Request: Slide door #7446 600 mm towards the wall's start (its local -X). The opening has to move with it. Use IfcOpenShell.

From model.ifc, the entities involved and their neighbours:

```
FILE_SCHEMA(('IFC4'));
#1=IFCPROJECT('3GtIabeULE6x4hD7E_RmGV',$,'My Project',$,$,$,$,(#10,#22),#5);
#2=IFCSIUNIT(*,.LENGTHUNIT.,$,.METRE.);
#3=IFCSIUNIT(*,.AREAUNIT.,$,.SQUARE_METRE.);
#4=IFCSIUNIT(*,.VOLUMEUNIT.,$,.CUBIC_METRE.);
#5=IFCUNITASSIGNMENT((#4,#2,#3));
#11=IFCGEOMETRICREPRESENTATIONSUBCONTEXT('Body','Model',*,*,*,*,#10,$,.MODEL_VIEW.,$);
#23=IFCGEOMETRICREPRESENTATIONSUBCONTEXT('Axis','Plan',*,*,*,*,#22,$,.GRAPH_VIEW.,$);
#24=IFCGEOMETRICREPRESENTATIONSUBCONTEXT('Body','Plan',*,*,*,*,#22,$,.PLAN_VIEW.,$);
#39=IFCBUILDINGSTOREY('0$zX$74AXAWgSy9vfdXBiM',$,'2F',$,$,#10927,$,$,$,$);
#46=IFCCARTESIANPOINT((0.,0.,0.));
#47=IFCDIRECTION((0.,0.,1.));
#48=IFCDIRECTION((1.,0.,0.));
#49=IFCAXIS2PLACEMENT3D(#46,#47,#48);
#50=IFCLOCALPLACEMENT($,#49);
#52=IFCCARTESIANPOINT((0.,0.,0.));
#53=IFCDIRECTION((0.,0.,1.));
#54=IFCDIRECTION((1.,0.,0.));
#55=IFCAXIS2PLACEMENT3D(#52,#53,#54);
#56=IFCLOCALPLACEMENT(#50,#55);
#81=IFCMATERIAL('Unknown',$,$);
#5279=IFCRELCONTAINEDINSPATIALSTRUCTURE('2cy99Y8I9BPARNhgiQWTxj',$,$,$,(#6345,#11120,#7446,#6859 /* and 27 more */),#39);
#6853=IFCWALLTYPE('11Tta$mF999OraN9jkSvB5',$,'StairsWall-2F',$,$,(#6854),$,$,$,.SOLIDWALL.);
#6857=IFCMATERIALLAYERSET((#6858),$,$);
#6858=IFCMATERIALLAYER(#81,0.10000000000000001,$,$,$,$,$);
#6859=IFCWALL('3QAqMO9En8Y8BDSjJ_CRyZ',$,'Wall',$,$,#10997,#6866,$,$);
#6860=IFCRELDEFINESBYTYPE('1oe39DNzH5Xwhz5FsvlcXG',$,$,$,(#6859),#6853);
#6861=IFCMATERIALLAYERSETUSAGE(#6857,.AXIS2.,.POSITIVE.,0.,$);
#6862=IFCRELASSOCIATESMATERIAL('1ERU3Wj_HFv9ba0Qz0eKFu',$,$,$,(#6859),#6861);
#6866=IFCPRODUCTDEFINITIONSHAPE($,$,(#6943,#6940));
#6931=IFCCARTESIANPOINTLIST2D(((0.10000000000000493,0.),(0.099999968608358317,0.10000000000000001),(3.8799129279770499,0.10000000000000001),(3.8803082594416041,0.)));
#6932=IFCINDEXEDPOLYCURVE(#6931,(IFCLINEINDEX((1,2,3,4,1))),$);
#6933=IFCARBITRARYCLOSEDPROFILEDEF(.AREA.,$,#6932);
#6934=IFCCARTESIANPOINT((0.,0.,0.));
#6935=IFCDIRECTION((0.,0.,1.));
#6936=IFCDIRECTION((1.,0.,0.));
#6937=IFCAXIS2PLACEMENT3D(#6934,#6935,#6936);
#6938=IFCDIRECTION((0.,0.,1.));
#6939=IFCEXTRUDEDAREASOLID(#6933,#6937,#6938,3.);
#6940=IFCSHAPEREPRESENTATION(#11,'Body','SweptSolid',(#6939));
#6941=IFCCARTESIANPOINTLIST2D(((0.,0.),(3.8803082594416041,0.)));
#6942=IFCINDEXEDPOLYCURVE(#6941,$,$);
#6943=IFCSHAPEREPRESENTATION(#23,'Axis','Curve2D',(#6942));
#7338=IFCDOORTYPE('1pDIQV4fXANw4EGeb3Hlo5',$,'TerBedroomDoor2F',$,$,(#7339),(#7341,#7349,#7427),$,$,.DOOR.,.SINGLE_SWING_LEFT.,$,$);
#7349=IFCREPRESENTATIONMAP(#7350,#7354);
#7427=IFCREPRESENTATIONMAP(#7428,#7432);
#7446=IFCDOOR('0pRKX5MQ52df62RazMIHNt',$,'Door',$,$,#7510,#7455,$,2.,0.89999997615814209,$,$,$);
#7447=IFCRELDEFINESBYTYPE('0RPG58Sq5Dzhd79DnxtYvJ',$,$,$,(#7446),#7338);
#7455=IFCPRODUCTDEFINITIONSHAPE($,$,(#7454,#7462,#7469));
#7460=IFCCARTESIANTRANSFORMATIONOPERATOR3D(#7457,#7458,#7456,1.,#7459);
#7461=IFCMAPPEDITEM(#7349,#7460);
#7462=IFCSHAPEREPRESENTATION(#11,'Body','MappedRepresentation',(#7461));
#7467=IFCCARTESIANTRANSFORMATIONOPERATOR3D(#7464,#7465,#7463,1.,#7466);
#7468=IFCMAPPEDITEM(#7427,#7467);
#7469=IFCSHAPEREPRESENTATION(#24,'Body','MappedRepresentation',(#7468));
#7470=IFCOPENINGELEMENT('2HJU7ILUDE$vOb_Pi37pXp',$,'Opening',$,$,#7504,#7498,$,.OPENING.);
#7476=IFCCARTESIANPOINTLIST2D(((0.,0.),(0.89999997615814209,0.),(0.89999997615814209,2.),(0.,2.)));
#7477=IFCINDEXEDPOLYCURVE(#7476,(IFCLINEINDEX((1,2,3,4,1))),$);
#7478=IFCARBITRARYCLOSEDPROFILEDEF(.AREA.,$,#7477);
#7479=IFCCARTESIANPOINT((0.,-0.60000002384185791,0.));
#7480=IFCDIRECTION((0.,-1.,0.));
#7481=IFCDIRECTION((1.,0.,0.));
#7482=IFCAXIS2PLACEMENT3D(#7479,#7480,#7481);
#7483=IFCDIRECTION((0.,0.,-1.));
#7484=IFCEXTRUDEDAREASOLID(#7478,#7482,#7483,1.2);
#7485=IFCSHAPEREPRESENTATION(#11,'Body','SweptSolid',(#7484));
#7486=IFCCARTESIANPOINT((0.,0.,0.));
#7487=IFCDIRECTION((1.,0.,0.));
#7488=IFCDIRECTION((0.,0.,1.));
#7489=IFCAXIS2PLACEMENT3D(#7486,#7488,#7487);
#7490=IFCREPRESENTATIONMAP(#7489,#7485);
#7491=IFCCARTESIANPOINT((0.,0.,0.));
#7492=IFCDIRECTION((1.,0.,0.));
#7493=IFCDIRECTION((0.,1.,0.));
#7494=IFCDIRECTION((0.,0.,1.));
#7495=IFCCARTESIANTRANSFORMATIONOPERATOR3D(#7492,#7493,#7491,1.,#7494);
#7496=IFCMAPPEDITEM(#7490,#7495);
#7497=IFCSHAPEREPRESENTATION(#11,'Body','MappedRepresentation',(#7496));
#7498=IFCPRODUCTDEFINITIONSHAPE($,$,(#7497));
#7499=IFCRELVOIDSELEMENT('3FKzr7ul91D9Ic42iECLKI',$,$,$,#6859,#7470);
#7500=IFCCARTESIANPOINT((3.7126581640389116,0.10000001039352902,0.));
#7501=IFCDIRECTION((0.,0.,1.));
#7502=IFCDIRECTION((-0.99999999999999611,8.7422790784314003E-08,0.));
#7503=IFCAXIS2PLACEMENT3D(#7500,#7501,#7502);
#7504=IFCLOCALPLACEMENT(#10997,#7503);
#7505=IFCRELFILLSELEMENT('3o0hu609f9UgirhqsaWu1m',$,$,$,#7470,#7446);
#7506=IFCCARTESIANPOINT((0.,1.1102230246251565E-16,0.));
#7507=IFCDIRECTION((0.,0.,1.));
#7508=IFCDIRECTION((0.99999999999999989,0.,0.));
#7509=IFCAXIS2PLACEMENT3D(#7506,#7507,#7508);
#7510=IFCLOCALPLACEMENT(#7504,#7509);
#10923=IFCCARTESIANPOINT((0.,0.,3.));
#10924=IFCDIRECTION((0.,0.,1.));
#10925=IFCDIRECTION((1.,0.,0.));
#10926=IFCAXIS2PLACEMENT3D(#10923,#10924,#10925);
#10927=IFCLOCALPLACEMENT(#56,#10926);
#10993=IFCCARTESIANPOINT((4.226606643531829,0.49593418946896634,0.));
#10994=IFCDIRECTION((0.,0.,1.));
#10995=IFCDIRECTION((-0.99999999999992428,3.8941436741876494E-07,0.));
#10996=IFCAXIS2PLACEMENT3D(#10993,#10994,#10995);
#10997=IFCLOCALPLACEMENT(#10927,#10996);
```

```python
import ifcopenshell
import ifcopenshell.api.geometry
import ifcopenshell.util.placement

model = ifcopenshell.open("model.ifc")

door = model.by_guid("0pRKX5MQ52df62RazMIHNt")
opening = door.FillsVoids[0].RelatingOpeningElement
wall = opening.VoidsElements[0].RelatingBuildingElement

wall_matrix = ifcopenshell.util.placement.get_local_placement(wall.ObjectPlacement)
shift = wall_matrix[:3, 0] * -0.6
before = ifcopenshell.util.placement.get_local_placement(door.ObjectPlacement)[:3, 3].copy()

# The door is placed relative to its opening, so it follows when the opening moves.
matrix = ifcopenshell.util.placement.get_local_placement(opening.ObjectPlacement)
matrix[:3, 3] += shift
ifcopenshell.api.geometry.edit_object_placement(
    model, product=opening, matrix=matrix, is_si=False, should_transform_children=True
)

after = ifcopenshell.util.placement.get_local_placement(door.ObjectPlacement)[:3, 3]
print("door moved by", (after - before).round(3) + 0.0)

model.write("model_v2.ifc")
```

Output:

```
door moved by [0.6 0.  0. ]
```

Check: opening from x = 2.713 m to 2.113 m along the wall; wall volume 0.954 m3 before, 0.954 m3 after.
